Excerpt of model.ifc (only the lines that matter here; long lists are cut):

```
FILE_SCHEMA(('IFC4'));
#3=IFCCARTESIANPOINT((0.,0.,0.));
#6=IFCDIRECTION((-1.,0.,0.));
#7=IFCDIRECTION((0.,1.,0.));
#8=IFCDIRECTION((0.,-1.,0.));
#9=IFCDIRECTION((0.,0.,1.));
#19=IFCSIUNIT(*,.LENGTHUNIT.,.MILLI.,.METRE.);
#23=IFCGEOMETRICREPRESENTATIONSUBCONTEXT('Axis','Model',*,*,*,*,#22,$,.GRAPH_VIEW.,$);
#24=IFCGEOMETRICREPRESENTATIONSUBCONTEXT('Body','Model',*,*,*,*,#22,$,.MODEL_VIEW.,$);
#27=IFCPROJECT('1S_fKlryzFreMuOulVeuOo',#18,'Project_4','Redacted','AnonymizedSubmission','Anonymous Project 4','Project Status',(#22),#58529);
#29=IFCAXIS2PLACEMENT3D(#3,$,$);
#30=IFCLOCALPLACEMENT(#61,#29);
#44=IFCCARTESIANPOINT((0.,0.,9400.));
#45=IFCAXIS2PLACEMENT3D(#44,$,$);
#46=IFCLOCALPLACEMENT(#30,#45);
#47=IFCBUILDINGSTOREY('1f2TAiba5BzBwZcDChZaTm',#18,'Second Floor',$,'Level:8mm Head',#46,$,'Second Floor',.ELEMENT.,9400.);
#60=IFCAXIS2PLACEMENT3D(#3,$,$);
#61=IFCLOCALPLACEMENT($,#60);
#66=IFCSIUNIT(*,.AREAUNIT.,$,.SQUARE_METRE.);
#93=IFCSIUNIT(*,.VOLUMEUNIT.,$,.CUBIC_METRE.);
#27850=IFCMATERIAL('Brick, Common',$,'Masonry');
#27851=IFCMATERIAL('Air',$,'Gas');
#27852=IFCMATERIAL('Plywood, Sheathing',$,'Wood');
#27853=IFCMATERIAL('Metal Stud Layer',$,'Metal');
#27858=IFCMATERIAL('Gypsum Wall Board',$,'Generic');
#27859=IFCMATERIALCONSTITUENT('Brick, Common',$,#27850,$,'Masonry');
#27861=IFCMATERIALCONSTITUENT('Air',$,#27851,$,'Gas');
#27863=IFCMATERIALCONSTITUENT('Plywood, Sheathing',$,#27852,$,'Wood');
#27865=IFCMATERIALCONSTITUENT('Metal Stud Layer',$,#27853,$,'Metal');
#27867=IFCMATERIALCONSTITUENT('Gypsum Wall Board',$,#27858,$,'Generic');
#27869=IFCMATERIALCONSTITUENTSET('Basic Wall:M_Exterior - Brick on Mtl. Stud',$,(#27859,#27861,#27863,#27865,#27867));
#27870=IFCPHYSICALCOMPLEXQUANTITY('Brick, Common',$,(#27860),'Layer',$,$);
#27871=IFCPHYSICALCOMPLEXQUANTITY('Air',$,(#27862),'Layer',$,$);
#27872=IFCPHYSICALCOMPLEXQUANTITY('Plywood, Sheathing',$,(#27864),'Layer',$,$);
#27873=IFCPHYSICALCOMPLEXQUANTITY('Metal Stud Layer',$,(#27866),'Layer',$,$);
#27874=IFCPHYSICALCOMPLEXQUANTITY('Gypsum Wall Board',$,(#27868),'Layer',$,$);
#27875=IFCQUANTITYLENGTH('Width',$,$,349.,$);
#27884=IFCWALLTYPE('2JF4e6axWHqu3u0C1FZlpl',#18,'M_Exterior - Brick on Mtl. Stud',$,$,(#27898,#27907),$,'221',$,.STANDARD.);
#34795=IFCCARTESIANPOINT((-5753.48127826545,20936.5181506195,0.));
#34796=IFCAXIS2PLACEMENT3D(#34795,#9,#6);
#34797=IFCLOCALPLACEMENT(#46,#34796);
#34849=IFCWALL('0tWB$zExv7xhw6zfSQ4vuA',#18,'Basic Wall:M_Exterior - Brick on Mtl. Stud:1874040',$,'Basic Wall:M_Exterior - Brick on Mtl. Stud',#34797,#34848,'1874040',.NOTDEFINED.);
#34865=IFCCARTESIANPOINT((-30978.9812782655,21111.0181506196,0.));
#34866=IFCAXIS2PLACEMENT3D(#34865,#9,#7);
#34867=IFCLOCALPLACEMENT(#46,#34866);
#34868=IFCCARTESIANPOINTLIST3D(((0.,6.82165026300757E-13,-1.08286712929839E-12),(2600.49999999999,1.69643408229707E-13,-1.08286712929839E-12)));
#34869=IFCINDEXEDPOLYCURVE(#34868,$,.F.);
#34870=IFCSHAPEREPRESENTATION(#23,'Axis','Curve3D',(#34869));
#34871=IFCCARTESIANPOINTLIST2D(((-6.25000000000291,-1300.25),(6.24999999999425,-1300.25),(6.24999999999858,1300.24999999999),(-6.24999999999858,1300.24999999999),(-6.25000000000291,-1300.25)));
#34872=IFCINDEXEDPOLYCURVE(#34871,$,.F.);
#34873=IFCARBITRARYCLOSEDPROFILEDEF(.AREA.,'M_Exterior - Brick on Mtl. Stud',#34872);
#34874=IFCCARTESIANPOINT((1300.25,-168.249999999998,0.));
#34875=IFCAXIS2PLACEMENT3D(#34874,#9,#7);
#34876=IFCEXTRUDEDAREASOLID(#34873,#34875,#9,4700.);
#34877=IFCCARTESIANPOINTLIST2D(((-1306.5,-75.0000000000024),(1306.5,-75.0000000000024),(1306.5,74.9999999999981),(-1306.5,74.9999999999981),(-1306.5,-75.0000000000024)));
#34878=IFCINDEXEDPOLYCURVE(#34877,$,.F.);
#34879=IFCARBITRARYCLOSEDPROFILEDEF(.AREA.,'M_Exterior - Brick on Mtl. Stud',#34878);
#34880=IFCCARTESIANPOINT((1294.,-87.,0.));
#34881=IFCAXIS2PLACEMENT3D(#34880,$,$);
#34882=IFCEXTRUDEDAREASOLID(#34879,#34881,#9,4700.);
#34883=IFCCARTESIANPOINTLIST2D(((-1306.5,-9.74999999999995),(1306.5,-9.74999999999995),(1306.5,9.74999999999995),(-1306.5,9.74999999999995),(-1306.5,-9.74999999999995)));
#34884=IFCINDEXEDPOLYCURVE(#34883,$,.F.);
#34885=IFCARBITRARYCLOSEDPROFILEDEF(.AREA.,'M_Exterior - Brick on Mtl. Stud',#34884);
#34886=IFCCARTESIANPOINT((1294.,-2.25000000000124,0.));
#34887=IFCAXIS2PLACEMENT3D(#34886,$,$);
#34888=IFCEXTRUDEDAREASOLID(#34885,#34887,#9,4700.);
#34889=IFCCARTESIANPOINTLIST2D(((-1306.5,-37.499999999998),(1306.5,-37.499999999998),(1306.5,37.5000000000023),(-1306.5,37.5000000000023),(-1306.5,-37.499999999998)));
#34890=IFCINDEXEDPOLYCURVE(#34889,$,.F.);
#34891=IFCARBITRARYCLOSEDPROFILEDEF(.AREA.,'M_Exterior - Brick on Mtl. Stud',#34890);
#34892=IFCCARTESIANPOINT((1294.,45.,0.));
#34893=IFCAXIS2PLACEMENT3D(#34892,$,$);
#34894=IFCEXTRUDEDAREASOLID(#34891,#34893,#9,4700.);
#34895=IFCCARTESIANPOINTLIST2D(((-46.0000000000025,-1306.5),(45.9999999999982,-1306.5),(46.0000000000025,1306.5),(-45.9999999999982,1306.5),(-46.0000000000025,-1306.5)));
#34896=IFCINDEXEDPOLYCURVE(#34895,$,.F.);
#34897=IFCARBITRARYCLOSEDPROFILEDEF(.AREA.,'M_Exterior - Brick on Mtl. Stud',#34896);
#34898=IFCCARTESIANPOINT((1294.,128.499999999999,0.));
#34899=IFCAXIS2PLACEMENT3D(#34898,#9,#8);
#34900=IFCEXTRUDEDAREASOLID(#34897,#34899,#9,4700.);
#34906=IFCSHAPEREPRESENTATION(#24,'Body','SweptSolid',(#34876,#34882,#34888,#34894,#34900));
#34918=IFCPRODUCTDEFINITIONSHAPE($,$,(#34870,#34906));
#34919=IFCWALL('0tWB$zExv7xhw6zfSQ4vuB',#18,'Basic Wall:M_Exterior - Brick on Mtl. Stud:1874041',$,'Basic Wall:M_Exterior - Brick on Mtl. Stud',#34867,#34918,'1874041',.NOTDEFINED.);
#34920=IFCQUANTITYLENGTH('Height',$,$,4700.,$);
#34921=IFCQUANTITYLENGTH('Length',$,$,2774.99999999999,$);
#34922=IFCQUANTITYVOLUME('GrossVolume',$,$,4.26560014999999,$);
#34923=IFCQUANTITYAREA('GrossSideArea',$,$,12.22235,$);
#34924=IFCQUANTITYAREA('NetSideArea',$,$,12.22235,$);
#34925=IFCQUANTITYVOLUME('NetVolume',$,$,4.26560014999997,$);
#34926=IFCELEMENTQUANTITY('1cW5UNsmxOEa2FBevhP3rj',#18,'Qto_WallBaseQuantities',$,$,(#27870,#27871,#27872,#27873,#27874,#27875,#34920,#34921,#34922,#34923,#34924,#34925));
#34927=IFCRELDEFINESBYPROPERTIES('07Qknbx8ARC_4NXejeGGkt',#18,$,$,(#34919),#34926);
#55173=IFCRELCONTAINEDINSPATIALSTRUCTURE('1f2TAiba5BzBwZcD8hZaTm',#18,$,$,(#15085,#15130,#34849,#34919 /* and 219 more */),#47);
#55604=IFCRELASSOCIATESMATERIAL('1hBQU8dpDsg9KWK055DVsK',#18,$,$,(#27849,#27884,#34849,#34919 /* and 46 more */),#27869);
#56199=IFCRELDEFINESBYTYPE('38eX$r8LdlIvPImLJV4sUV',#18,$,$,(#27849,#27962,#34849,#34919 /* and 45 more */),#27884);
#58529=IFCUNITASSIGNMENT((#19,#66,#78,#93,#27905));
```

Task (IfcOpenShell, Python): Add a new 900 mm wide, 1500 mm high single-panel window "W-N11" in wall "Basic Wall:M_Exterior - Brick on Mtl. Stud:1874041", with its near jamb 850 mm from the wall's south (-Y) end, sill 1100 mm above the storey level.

```python
import numpy as np
import ifcopenshell
import ifcopenshell.api.feature
import ifcopenshell.api.geometry
import ifcopenshell.api.pset
import ifcopenshell.api.root
import ifcopenshell.api.spatial
import ifcopenshell.geom
import ifcopenshell.util.element
import ifcopenshell.util.placement
import ifcopenshell.util.representation
import ifcopenshell.util.shape
import ifcopenshell.util.unit

model = ifcopenshell.open("model.ifc")
unit_scale = ifcopenshell.util.unit.calculate_unit_scale(model)
area_scale = ifcopenshell.util.unit.calculate_unit_scale(model, "AREAUNIT")
volume_scale = ifcopenshell.util.unit.calculate_unit_scale(model, "VOLUMEUNIT")
settings = ifcopenshell.geom.settings()


def volume(element):
    """Net volume in cubic metres, openings subtracted."""
    shape = ifcopenshell.geom.create_shape(settings, element)
    return ifcopenshell.util.shape.get_volume(shape.geometry)


wall = model.by_id(34919)
storey = ifcopenshell.util.element.get_container(wall, ifc_class="IfcBuildingStorey")
context = ifcopenshell.util.representation.get_context(model, "Model", "Body", "MODEL_VIEW")
before = volume(wall)

width, height, from_end, sill = 0.9, 1.5, 0.85, 1.1  # metres

# The wall runs along its own X axis, and the end named is its -X end.
wall_shape = ifcopenshell.geom.create_shape(settings, wall)
x, y, z = ifcopenshell.util.shape.get_vertices(wall_shape.geometry).T
start = x.min() + from_end
face, thickness = float(y.min()), float(y.max() - y.min())
wall_matrix = ifcopenshell.util.placement.get_local_placement(wall.ObjectPlacement)
level = ifcopenshell.util.placement.get_local_placement(storey.ObjectPlacement)[2, 3]


def in_wall(x, y):
    """Placement at x, y metres in the wall's axes, at sill height."""
    matrix = wall_matrix.copy()
    matrix[:, 3] = wall_matrix @ np.array([x / unit_scale, y / unit_scale, 0.0, 1.0])
    matrix[2, 3] = level + sill / unit_scale
    return matrix


# Opening: a box that overshoots both wall faces by 50 mm.
opening = ifcopenshell.api.root.create_entity(model, ifc_class="IfcOpeningElement", predefined_type="OPENING")
box = ifcopenshell.api.geometry.add_wall_representation(
    model, context=context, length=width, height=height, thickness=thickness + 0.1
)
ifcopenshell.api.geometry.assign_representation(model, product=opening, representation=box)
ifcopenshell.api.geometry.edit_object_placement(model, product=opening, matrix=in_wall(start, face - 0.05), is_si=False)
ifcopenshell.api.feature.add_feature(model, feature=opening, element=wall)

window = ifcopenshell.api.root.create_entity(model, ifc_class="IfcWindow", name="W-N11", predefined_type="WINDOW")
window.OverallWidth, window.OverallHeight = width / unit_scale, height / unit_scale
window.PartitioningType = "SINGLE_PANEL"
body = ifcopenshell.api.geometry.add_window_representation(
    model,
    context=context,
    overall_width=window.OverallWidth,
    overall_height=window.OverallHeight,
    partition_type="SINGLE_PANEL",
)
ifcopenshell.api.geometry.assign_representation(model, product=window, representation=body)
ifcopenshell.api.spatial.assign_container(model, products=[window], relating_structure=storey)
ifcopenshell.api.feature.add_filling(model, opening=opening, element=window)

# Centre the window in the wall's thickness.
ifcopenshell.api.geometry.edit_object_placement(model, product=window, matrix=in_wall(start, face), is_si=False)
window_shape = ifcopenshell.geom.create_shape(settings, window)
depth = ifcopenshell.util.shape.get_vertices(window_shape.geometry)[:, 1]
offset = face + thickness / 2 - (depth.min() + depth.max()) / 2
ifcopenshell.api.geometry.edit_object_placement(model, product=window, matrix=in_wall(start, offset), is_si=False)

after = volume(wall)

# Update the wall's stored quantities.
qto = model.by_id(ifcopenshell.util.element.get_pset(wall, "Qto_WallBaseQuantities", should_inherit=False)["id"])
ifcopenshell.api.pset.edit_qto(model, qto=qto, properties={
    "NetSideArea": after / thickness / area_scale,
    "NetVolume": after / volume_scale,
})

print(f"wall volume {before:.3f} -> {after:.3f} m3")

model.write("model_updated.ifc")
```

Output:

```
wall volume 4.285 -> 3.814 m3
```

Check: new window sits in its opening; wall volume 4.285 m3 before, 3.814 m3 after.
